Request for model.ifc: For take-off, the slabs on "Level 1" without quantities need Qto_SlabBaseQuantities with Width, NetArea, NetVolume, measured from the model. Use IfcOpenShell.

First a look at what the model holds.

```python
import ifcopenshell
import ifcopenshell.util.element
import ifcopenshell.util.unit

model = ifcopenshell.open("model.ifc")
print(model.schema)
for unit_type in ("LENGTHUNIT", "AREAUNIT", "VOLUMEUNIT"):
    print(unit_type, ifcopenshell.util.unit.calculate_unit_scale(model, unit_type))
storey = next(s for s in model.by_type("IfcBuildingStorey") if s.Name == "Level 1")
slabs = [e for e in ifcopenshell.util.element.get_decomposition(storey) if e.is_a("IfcSlab")]
for e in sorted(slabs, key=lambda e: e.id()):
    print(e.id(), e.is_a(), e.Name, list(ifcopenshell.util.element.get_psets(e, qtos_only=True)), sep=" | ")
```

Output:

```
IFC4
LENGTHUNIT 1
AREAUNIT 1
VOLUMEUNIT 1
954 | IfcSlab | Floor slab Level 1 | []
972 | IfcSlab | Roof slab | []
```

```python
import ifcopenshell
import ifcopenshell.api.pset
import ifcopenshell.geom
import ifcopenshell.util.element
import ifcopenshell.util.shape
import ifcopenshell.util.unit

model = ifcopenshell.open("model.ifc")
unit_scale = ifcopenshell.util.unit.calculate_unit_scale(model)
area_scale = ifcopenshell.util.unit.calculate_unit_scale(model, "AREAUNIT")
volume_scale = ifcopenshell.util.unit.calculate_unit_scale(model, "VOLUMEUNIT")
settings = ifcopenshell.geom.settings()

storey = next(s for s in model.by_type("IfcBuildingStorey") if s.Name == "Level 1")
slabs = [e for e in ifcopenshell.util.element.get_decomposition(storey) if e.is_a("IfcSlab")]

for e in sorted(slabs, key=lambda e: e.id()):
    if ifcopenshell.util.element.get_psets(e, qtos_only=True, should_inherit=False):
        continue
    # Geometry comes back in metres, in the element's own axes.
    shape = ifcopenshell.geom.create_shape(settings, e)
    values = {
        "Width": ifcopenshell.util.shape.get_z(shape.geometry) / unit_scale,
        "NetArea": ifcopenshell.util.shape.get_footprint_area(shape.geometry) / area_scale,
        "NetVolume": ifcopenshell.util.shape.get_volume(shape.geometry) / volume_scale,
    }
    qto = ifcopenshell.api.pset.add_qto(model, product=e, name="Qto_SlabBaseQuantities")
    ifcopenshell.api.pset.edit_qto(model, qto=qto, properties=values)
    print(e.id(), {k: round(v, 3) for k, v in values.items()})

model.write("model_updated.ifc")
```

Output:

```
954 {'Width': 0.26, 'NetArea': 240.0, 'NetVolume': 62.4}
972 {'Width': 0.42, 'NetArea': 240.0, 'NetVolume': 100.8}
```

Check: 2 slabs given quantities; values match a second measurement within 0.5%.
